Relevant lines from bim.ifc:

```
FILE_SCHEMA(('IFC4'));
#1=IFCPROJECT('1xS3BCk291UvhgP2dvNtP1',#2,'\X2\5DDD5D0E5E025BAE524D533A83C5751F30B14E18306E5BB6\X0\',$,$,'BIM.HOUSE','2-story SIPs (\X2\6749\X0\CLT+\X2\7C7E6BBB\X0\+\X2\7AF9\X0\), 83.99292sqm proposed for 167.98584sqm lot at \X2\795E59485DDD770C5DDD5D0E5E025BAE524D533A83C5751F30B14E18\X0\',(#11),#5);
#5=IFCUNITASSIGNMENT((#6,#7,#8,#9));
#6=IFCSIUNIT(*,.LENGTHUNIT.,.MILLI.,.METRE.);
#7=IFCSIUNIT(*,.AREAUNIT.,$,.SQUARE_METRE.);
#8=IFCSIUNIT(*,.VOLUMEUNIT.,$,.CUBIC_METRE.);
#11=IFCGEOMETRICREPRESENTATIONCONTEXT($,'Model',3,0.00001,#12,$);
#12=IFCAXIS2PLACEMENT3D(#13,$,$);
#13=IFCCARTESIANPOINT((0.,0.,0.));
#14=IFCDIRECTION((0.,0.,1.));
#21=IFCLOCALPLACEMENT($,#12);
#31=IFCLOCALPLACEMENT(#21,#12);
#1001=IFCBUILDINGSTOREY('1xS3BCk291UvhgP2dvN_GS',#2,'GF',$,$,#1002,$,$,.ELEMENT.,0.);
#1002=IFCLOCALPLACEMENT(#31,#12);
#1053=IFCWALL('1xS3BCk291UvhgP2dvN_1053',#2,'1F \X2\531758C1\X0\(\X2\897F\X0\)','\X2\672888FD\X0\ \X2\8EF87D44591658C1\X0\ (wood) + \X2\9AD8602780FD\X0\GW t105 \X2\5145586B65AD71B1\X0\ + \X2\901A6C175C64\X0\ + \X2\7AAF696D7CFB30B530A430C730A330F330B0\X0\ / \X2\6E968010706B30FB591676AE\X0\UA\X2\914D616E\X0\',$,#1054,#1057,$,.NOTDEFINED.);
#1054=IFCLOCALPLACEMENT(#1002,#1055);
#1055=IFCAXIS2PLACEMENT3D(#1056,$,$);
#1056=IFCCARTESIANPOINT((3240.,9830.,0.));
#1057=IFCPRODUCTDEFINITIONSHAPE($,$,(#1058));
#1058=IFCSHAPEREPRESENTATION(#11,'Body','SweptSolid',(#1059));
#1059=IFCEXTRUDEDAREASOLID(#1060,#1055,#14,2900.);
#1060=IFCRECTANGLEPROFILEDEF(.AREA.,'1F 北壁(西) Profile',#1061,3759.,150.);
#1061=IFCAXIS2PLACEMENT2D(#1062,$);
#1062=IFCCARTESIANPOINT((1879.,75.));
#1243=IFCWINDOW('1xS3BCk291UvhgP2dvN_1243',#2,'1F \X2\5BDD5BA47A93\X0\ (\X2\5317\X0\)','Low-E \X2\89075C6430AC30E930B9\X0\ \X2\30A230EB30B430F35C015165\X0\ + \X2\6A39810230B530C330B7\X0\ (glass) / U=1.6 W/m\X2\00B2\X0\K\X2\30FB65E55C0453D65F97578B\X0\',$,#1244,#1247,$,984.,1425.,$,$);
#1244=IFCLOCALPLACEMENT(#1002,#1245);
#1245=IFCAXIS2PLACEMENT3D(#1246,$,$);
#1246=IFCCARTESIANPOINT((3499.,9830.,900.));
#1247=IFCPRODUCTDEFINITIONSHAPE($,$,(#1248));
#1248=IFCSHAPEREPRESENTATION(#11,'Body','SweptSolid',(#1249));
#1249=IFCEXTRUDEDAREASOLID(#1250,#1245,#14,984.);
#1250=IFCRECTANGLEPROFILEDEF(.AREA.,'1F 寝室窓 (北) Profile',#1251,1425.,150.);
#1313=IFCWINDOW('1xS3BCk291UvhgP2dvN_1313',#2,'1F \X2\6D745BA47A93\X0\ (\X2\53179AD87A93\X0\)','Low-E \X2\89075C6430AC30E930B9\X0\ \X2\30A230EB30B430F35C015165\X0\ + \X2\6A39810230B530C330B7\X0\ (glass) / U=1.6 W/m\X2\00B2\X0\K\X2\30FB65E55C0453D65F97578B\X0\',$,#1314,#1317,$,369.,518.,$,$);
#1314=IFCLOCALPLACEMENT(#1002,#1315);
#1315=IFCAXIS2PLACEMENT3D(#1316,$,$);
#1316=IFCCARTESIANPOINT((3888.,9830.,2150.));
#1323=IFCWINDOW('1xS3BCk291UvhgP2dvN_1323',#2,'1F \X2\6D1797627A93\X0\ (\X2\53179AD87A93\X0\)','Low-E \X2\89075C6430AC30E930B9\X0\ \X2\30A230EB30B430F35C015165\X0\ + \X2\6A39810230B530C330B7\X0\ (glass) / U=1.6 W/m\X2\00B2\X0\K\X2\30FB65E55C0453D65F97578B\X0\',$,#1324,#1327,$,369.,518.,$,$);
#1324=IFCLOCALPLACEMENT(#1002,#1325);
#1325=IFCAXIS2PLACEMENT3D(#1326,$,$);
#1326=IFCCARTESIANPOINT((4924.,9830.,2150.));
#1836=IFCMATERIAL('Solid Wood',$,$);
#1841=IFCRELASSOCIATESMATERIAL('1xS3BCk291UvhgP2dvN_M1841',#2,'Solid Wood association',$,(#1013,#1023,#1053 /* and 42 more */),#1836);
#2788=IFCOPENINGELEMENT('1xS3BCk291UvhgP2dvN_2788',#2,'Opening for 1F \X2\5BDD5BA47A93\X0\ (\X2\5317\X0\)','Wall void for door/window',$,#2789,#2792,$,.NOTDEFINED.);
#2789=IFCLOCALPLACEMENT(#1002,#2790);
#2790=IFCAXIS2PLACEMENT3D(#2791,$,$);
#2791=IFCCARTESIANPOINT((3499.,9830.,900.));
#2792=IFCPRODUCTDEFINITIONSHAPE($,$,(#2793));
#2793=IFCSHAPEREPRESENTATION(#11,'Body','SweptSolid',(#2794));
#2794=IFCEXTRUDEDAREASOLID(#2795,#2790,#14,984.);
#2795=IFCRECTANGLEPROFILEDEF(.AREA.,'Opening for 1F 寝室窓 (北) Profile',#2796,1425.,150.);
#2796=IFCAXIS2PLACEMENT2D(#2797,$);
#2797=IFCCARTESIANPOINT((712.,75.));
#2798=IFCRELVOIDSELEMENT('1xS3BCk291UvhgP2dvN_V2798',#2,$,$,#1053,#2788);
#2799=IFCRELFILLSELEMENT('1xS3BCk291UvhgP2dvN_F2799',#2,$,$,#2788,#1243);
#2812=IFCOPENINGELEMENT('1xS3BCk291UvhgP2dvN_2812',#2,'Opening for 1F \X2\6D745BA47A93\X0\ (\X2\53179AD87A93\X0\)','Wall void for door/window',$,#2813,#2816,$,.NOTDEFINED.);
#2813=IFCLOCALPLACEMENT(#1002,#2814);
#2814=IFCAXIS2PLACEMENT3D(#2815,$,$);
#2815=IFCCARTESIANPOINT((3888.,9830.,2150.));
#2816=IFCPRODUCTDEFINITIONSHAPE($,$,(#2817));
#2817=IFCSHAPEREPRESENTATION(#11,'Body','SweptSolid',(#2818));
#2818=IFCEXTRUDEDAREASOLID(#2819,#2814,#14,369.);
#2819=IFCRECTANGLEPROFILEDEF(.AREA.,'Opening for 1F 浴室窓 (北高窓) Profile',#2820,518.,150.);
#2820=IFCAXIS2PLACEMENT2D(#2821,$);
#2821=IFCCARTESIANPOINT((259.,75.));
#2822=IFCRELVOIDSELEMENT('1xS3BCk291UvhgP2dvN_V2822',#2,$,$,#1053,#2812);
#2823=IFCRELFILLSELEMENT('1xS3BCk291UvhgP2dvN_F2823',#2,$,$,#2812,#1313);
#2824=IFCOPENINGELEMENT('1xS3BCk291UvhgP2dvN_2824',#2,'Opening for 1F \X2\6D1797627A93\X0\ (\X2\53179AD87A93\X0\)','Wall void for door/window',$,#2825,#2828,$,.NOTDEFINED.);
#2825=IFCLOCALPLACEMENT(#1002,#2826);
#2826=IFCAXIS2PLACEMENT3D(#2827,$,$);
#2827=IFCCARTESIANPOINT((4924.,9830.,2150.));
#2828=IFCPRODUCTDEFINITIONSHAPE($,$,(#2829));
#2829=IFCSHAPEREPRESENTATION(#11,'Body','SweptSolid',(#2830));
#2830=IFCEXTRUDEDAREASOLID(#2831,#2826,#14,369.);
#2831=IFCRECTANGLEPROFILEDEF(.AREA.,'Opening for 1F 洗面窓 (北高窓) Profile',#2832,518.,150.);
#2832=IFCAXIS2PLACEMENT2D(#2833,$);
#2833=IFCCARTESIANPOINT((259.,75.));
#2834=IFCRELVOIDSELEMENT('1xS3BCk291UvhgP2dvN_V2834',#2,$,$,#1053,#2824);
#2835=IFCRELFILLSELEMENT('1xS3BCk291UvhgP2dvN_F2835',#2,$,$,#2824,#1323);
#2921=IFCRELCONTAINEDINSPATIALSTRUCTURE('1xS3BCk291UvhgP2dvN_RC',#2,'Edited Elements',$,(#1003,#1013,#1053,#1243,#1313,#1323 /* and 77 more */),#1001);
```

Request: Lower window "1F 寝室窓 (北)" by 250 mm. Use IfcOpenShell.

```python
import numpy as np
import ifcopenshell
import ifcopenshell.api.geometry
import ifcopenshell.util.placement
import ifcopenshell.util.unit

model = ifcopenshell.open("bim.ifc")
unit_scale = ifcopenshell.util.unit.calculate_unit_scale(model)

window = model.by_guid("1xS3BCk291UvhgP2dvN_1243")
opening = window.FillsVoids[0].RelatingOpeningElement
dz = -250.0

shift = np.array([0.0, 0.0, dz])
# The window is not placed relative to its opening, so move both.
for product in (opening, window):
    matrix = ifcopenshell.util.placement.get_local_placement(product.ObjectPlacement)
    matrix[:3, 3] += shift
    ifcopenshell.api.geometry.edit_object_placement(model, product=product, matrix=matrix, is_si=False)

print(f"moved by {dz * unit_scale:+.3f} m")

model.write("bim_edited.ifc")
```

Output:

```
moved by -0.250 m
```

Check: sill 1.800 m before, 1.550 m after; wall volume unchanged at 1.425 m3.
